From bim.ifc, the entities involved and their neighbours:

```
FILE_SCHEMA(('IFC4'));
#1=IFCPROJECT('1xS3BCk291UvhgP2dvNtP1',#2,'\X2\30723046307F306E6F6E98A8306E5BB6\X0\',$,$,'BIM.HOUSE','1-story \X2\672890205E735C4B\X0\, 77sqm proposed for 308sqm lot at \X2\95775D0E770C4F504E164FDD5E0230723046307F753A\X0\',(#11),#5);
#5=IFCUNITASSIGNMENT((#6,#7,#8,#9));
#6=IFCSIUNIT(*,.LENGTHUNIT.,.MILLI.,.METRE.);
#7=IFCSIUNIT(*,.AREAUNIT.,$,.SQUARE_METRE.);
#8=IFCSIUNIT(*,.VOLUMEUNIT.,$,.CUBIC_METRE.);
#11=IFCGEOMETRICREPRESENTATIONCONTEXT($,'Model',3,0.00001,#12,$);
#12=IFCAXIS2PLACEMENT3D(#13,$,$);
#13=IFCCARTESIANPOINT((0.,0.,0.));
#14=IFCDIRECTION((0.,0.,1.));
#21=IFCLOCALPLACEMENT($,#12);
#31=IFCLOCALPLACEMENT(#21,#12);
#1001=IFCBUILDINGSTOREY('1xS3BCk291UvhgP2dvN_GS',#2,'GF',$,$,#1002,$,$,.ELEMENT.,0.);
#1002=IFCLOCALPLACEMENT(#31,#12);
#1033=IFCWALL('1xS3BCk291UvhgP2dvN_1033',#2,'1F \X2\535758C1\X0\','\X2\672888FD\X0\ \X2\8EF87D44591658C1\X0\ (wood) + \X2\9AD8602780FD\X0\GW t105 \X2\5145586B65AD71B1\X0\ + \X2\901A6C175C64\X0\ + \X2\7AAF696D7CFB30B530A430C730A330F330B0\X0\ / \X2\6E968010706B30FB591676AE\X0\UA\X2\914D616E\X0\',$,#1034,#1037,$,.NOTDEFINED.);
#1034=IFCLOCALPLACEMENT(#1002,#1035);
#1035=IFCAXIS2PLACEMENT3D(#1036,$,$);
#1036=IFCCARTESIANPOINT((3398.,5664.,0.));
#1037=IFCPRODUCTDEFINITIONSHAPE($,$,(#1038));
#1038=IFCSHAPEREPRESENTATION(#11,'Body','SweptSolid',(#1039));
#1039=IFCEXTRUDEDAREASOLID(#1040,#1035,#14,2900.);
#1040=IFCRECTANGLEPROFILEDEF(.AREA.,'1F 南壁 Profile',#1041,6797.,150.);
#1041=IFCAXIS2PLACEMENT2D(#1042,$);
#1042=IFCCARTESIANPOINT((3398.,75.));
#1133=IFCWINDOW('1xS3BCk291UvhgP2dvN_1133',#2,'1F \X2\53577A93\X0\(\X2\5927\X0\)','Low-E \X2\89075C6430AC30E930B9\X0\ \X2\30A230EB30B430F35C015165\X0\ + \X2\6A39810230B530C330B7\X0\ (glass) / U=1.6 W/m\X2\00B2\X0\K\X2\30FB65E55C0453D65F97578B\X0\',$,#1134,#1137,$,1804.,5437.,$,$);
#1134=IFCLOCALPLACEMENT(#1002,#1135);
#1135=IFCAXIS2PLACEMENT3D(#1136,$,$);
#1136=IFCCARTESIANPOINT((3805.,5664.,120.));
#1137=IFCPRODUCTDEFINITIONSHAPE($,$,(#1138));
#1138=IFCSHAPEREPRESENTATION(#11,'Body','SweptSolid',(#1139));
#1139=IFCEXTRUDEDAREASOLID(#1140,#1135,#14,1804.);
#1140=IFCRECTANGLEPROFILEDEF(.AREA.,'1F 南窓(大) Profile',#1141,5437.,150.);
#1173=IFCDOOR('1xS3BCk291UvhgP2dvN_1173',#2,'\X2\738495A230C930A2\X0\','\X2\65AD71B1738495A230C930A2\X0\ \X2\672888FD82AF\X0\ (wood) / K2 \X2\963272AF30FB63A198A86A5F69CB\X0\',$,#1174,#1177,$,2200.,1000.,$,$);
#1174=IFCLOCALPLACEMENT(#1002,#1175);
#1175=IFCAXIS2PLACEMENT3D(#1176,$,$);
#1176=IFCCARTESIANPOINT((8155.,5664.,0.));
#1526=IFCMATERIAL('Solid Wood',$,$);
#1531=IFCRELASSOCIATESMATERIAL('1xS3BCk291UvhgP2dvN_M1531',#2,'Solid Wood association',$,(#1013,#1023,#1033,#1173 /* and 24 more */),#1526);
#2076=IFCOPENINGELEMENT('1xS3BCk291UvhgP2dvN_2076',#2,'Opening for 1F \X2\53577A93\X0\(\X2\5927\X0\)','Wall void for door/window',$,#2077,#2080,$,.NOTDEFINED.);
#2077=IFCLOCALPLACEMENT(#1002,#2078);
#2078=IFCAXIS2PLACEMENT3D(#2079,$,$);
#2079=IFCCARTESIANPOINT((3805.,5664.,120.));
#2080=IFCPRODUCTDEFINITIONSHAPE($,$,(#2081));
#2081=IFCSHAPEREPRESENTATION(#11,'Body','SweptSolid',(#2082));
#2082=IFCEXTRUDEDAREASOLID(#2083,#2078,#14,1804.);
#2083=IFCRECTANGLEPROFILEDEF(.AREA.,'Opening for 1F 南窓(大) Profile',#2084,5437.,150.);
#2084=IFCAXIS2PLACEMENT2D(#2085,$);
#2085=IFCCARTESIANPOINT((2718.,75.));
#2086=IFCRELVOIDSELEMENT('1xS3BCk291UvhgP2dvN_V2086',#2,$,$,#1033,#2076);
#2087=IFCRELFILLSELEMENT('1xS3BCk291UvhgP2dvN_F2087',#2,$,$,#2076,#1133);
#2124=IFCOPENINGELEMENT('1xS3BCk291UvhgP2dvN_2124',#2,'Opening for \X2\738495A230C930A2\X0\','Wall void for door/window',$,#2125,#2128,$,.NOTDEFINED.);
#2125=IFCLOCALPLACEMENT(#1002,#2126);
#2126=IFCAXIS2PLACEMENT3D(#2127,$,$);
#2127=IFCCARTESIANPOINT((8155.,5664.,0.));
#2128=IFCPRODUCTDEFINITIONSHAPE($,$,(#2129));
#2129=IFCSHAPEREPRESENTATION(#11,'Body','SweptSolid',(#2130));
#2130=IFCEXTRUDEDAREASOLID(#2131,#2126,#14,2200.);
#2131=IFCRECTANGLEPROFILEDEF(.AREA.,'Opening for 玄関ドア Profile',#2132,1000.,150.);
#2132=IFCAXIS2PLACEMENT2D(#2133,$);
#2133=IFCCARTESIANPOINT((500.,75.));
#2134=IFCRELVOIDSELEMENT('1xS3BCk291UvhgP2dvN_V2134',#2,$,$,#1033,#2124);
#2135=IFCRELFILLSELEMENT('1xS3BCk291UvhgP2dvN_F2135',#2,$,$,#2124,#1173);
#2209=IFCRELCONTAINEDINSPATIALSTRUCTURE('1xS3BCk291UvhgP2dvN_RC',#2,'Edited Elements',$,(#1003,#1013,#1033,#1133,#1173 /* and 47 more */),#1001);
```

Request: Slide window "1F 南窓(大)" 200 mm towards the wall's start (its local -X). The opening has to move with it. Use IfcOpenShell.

```python
import ifcopenshell
import ifcopenshell.api.geometry
import ifcopenshell.util.placement
import ifcopenshell.util.unit

model = ifcopenshell.open("bim.ifc")
unit_scale = ifcopenshell.util.unit.calculate_unit_scale(model)

window = model.by_id(1133)
opening = window.FillsVoids[0].RelatingOpeningElement
wall = opening.VoidsElements[0].RelatingBuildingElement

wall_matrix = ifcopenshell.util.placement.get_local_placement(wall.ObjectPlacement)
shift = wall_matrix[:3, 0] * -0.2 / unit_scale
before = ifcopenshell.util.placement.get_local_placement(window.ObjectPlacement)[:3, 3].copy()

# The window is not placed relative to its opening, so move both.
for product in (opening, window):
    matrix = ifcopenshell.util.placement.get_local_placement(product.ObjectPlacement)
    matrix[:3, 3] += shift
    ifcopenshell.api.geometry.edit_object_placement(model, product=product, matrix=matrix, is_si=False)

after = ifcopenshell.util.placement.get_local_placement(window.ObjectPlacement)[:3, 3]
print("window moved by", (after - before).round(3) + 0.0)

model.write("bim_updated.ifc")
```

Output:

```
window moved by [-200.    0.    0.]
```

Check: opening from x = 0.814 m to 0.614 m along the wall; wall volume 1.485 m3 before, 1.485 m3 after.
